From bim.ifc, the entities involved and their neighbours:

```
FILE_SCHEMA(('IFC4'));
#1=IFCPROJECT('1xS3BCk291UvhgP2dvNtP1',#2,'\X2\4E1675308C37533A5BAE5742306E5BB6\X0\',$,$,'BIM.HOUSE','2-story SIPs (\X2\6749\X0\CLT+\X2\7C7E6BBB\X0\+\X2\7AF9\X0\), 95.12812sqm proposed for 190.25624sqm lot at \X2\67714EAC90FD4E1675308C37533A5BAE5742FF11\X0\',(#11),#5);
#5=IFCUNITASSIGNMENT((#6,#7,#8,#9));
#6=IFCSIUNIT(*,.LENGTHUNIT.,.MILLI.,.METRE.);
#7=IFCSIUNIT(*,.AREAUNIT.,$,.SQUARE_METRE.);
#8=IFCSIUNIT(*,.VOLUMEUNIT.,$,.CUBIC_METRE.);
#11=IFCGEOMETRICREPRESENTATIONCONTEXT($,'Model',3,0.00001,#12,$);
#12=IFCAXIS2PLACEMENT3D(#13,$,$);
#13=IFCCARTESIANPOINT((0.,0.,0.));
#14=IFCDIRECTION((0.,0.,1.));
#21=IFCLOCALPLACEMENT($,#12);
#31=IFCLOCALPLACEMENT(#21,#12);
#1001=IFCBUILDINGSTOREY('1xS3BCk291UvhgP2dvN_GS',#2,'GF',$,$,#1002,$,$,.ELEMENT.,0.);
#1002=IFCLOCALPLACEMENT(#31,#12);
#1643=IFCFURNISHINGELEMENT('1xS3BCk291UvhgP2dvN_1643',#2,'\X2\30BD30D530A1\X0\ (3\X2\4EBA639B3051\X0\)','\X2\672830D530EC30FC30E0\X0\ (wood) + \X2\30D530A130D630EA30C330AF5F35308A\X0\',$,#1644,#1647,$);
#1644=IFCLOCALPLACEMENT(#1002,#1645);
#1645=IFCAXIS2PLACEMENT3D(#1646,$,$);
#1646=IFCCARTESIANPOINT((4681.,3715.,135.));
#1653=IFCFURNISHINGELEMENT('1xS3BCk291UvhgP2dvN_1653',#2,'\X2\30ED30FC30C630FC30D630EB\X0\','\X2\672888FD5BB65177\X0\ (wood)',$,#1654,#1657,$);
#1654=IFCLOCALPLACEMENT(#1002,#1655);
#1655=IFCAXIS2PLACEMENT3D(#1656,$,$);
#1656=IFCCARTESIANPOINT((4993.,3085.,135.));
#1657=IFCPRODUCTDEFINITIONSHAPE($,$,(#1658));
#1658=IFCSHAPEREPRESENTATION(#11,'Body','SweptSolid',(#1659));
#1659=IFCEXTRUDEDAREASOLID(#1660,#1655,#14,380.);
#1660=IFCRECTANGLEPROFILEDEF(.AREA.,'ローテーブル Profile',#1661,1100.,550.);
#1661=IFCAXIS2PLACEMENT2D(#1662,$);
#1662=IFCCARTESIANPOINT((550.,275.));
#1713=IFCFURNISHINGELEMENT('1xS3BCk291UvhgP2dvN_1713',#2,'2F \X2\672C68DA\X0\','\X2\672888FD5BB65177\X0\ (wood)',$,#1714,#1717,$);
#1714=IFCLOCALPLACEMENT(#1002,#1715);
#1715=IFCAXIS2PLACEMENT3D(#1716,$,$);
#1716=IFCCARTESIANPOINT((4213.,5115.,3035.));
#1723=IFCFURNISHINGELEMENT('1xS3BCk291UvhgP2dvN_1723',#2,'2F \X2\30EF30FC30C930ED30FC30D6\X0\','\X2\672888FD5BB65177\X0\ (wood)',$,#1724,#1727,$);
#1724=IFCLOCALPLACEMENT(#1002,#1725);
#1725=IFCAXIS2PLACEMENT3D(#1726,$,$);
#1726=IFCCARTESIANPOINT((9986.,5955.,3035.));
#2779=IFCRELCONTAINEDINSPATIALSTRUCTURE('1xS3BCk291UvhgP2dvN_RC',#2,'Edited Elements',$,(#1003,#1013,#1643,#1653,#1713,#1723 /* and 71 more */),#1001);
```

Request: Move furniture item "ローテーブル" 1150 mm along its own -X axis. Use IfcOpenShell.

```python
import ifcopenshell
import ifcopenshell.api.geometry
import ifcopenshell.util.placement
import ifcopenshell.util.unit

model = ifcopenshell.open("bim.ifc")
unit_scale = ifcopenshell.util.unit.calculate_unit_scale(model)

item = model.by_guid("1xS3BCk291UvhgP2dvN_1653")
matrix = ifcopenshell.util.placement.get_local_placement(item.ObjectPlacement)
matrix[:3, 3] -= matrix[:3, 0] * 1.15 / unit_scale
ifcopenshell.api.geometry.edit_object_placement(model, product=item, matrix=matrix, is_si=False)

print(ifcopenshell.util.placement.get_local_placement(item.ObjectPlacement).round(3) + 0.0)

model.write("bim_edited.ifc")
```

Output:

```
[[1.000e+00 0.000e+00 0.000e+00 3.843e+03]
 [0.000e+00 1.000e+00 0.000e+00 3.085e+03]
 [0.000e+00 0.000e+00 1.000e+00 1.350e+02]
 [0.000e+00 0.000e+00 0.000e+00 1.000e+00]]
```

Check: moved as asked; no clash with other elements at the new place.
